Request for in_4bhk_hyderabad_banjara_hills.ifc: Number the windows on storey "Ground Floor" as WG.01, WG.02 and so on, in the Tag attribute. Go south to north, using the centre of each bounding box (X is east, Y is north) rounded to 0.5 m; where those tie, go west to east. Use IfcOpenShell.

First a look at what the model holds.

```python
import ifcopenshell
import ifcopenshell.util.element
import ifcopenshell.util.placement

model = ifcopenshell.open("in_4bhk_hyderabad_banjara_hills.ifc")
print(model.schema)
storey = next(s for s in model.by_type("IfcBuildingStorey") if s.Name == "Ground Floor")
windows = [e for e in ifcopenshell.util.element.get_decomposition(storey) if e.is_a("IfcWindow")]
for e in sorted(windows, key=lambda e: e.id()):
    origin = ifcopenshell.util.placement.get_local_placement(e.ObjectPlacement)[:3, 3]
    print(e.id(), e.Tag, e.Name, origin.round(2) + 0.0, sep=" | ")
```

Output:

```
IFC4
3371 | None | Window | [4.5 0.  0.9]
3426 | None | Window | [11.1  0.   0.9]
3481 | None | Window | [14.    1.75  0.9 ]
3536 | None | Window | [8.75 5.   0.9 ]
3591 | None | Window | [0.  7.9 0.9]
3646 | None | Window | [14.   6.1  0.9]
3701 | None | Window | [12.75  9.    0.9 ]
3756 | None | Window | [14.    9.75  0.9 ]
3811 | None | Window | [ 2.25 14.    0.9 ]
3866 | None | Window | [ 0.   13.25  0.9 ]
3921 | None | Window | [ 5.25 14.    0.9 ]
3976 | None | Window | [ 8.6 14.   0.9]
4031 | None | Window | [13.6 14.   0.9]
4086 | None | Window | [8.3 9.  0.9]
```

```python
import ifcopenshell
import ifcopenshell.geom
import ifcopenshell.util.element
import ifcopenshell.util.shape

model = ifcopenshell.open("in_4bhk_hyderabad_banjara_hills.ifc")
settings = ifcopenshell.geom.settings()
settings.set("use-world-coords", True)


def centre(element):
    shape = ifcopenshell.geom.create_shape(settings, element)
    return ifcopenshell.util.shape.get_bbox_centroid(shape.geometry)


storey = next(s for s in model.by_type("IfcBuildingStorey") if s.Name == "Ground Floor")
windows = [e for e in ifcopenshell.util.element.get_decomposition(storey) if e.is_a("IfcWindow")]

# Insertion points can sit at a corner or the storey origin, so sort by the geometry (in metres).
centres = {e: centre(e) for e in windows}
windows.sort(key=lambda e: (round(centres[e][1] / 0.5), centres[e][0]))

for i, e in enumerate(windows, start=1):
    number = f"WG.{i:02d}"
    e.Tag = number
    print(e.id(), number)

model.write("in_4bhk_hyderabad_banjara_hills_v2.ifc")
```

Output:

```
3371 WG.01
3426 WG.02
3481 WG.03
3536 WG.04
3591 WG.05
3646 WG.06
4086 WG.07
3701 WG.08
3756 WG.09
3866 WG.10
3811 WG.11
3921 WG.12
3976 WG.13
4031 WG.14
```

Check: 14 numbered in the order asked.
